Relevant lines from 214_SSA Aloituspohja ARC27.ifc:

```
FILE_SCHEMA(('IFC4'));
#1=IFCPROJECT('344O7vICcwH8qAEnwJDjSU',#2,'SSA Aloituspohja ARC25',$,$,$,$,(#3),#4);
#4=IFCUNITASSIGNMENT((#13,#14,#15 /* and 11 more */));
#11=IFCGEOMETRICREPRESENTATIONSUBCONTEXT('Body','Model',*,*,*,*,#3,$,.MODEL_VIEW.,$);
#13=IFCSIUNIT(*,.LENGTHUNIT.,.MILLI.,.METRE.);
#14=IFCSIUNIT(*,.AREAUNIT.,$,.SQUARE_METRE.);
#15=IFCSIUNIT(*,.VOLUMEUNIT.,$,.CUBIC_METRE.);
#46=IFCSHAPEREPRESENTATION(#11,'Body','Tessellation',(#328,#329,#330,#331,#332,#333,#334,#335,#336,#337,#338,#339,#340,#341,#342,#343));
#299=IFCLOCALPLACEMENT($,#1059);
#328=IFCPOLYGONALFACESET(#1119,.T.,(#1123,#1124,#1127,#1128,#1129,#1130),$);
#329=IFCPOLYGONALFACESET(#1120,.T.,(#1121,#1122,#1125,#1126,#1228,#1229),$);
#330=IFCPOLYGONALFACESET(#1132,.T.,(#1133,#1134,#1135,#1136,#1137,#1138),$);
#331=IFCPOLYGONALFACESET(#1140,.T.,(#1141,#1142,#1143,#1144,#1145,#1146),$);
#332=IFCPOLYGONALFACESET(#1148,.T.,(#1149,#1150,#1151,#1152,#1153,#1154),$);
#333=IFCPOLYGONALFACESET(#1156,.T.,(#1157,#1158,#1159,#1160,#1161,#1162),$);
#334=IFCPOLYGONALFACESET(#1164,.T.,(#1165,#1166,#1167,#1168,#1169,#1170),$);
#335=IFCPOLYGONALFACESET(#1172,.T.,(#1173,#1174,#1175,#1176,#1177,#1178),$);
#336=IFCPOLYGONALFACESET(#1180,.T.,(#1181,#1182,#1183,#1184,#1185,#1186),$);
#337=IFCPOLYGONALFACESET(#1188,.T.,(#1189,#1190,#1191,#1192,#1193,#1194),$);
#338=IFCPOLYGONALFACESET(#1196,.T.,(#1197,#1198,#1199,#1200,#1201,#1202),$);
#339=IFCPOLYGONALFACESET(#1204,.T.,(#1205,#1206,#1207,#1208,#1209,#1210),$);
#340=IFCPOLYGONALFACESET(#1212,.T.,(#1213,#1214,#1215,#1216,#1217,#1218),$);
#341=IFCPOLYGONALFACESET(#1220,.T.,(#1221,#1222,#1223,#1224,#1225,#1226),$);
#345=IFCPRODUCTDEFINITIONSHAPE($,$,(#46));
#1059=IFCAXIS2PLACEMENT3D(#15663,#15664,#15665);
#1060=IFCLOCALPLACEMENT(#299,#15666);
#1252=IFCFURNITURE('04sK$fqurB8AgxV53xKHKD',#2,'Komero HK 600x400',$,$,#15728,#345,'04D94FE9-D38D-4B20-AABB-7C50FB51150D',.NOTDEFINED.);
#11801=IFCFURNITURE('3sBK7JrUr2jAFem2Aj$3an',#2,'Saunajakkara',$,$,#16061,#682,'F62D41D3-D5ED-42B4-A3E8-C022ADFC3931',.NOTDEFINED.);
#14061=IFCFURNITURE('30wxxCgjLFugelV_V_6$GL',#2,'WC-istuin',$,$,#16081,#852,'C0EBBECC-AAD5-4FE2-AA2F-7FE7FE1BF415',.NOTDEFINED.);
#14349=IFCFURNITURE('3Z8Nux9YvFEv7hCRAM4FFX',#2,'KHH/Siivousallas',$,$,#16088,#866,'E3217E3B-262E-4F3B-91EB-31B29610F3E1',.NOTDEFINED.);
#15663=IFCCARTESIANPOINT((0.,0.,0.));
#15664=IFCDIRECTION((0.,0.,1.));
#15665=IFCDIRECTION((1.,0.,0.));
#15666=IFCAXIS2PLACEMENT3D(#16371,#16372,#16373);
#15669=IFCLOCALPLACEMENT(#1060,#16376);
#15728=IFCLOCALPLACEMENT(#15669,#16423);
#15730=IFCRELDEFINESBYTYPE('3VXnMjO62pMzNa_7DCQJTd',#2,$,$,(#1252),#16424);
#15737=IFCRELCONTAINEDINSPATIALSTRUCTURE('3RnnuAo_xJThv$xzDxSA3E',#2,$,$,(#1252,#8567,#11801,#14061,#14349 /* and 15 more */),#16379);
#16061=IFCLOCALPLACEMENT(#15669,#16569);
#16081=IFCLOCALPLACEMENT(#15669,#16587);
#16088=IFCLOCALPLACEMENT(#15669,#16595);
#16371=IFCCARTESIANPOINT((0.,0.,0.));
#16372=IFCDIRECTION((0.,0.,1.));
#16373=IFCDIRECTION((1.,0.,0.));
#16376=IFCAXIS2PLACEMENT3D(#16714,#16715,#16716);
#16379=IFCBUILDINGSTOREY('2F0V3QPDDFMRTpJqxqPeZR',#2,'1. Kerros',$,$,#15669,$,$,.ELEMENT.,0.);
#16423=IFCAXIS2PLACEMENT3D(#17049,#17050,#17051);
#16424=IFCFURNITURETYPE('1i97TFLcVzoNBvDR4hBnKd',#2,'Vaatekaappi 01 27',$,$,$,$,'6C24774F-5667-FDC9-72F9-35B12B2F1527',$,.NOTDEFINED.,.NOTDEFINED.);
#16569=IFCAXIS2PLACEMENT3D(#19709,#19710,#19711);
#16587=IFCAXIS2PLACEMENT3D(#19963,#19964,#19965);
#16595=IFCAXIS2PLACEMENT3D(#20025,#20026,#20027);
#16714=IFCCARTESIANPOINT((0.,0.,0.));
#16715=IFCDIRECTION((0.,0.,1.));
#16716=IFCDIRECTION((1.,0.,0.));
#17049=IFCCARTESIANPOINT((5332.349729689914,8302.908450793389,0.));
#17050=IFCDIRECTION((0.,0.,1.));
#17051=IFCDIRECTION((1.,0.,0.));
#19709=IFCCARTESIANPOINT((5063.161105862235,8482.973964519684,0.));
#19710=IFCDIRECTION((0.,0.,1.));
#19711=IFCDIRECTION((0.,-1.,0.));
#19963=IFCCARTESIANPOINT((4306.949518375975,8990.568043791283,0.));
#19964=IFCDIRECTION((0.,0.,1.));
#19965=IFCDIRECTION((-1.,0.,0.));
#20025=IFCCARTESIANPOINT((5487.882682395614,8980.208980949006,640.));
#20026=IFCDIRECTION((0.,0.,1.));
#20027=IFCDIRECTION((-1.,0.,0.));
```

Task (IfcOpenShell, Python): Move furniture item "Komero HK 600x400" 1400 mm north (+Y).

```python
import ifcopenshell
import ifcopenshell.api.geometry
import ifcopenshell.util.placement
import ifcopenshell.util.unit

model = ifcopenshell.open("214_SSA Aloituspohja ARC27.ifc")
unit_scale = ifcopenshell.util.unit.calculate_unit_scale(model)

item = model.by_id(1252)
matrix = ifcopenshell.util.placement.get_local_placement(item.ObjectPlacement)
matrix[1, 3] += 1.4 / unit_scale
ifcopenshell.api.geometry.edit_object_placement(model, product=item, matrix=matrix, is_si=False)

print(ifcopenshell.util.placement.get_local_placement(item.ObjectPlacement).round(3) + 0.0)

model.write("214_SSA Aloituspohja ARC27_updated.ifc")
```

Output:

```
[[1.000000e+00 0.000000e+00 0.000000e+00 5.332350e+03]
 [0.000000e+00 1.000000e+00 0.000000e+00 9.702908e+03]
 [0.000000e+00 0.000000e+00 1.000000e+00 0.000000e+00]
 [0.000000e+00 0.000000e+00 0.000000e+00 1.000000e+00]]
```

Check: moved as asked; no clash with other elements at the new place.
